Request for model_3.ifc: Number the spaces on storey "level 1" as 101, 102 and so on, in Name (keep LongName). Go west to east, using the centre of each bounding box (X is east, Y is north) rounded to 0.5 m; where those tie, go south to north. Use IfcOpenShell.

First a look at what the model holds.

```python
import ifcopenshell
import ifcopenshell.util.element
import ifcopenshell.util.placement

model = ifcopenshell.open("model_3.ifc")
print(model.schema)
storey = next(s for s in model.by_type("IfcBuildingStorey") if s.Name == "level 1")
spaces = [e for e in ifcopenshell.util.element.get_decomposition(storey) if e.is_a("IfcSpace")]
for e in sorted(spaces, key=lambda e: e.id()):
    origin = ifcopenshell.util.placement.get_local_placement(e.ObjectPlacement)[:3, 3]
    print(e.id(), e.Name, e.LongName, origin.round(2) + 0.0, sep=" | ")
```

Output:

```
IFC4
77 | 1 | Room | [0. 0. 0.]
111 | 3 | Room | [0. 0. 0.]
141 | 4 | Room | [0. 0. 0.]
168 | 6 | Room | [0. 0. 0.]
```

```python
import ifcopenshell
import ifcopenshell.geom
import ifcopenshell.util.element
import ifcopenshell.util.shape

model = ifcopenshell.open("model_3.ifc")
settings = ifcopenshell.geom.settings()
settings.set("use-world-coords", True)


def centre(element):
    shape = ifcopenshell.geom.create_shape(settings, element)
    return ifcopenshell.util.shape.get_bbox_centroid(shape.geometry)


storey = next(s for s in model.by_type("IfcBuildingStorey") if s.Name == "level 1")
spaces = [e for e in ifcopenshell.util.element.get_decomposition(storey) if e.is_a("IfcSpace")]

# Insertion points can sit at a corner or the storey origin, so sort by the geometry (in metres).
centres = {e: centre(e) for e in spaces}
spaces.sort(key=lambda e: (round(centres[e][0] / 0.5), centres[e][1]))

for i, e in enumerate(spaces, start=1):
    number = f"1{i:02d}"
    e.Name = number
    print(e.id(), number)

model.write("model_3_updated.ifc")
```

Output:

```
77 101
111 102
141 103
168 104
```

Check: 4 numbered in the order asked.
